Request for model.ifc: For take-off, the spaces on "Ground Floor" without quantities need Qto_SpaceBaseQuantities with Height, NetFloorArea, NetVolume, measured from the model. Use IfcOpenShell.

First a look at what the model holds.

```python
import ifcopenshell
import ifcopenshell.util.element
import ifcopenshell.util.unit

model = ifcopenshell.open("model.ifc")
print(model.schema)
for unit_type in ("LENGTHUNIT", "AREAUNIT", "VOLUMEUNIT"):
    print(unit_type, ifcopenshell.util.unit.calculate_unit_scale(model, unit_type))
storey = next(s for s in model.by_type("IfcBuildingStorey") if s.Name == "Ground Floor")
spaces = [e for e in ifcopenshell.util.element.get_decomposition(storey) if e.is_a("IfcSpace")]
for e in sorted(spaces, key=lambda e: e.id()):
    print(e.id(), e.is_a(), e.Name, list(ifcopenshell.util.element.get_psets(e, qtos_only=True)), sep=" | ")
```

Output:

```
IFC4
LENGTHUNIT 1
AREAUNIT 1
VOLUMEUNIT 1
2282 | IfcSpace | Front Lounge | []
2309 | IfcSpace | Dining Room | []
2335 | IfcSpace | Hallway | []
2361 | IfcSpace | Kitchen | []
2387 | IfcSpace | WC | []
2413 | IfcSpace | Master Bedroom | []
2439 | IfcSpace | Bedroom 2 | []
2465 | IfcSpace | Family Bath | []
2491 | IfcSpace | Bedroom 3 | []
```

```python
import ifcopenshell
import ifcopenshell.api.pset
import ifcopenshell.geom
import ifcopenshell.util.element
import ifcopenshell.util.shape
import ifcopenshell.util.unit

model = ifcopenshell.open("model.ifc")
unit_scale = ifcopenshell.util.unit.calculate_unit_scale(model)
area_scale = ifcopenshell.util.unit.calculate_unit_scale(model, "AREAUNIT")
volume_scale = ifcopenshell.util.unit.calculate_unit_scale(model, "VOLUMEUNIT")
settings = ifcopenshell.geom.settings()

storey = next(s for s in model.by_type("IfcBuildingStorey") if s.Name == "Ground Floor")
spaces = [e for e in ifcopenshell.util.element.get_decomposition(storey) if e.is_a("IfcSpace")]

for e in sorted(spaces, key=lambda e: e.id()):
    if ifcopenshell.util.element.get_psets(e, qtos_only=True, should_inherit=False):
        continue
    # Geometry comes back in metres, in the element's own axes.
    shape = ifcopenshell.geom.create_shape(settings, e)
    values = {
        "Height": ifcopenshell.util.shape.get_z(shape.geometry) / unit_scale,
        "NetFloorArea": ifcopenshell.util.shape.get_footprint_area(shape.geometry) / area_scale,
        "NetVolume": ifcopenshell.util.shape.get_volume(shape.geometry) / volume_scale,
    }
    qto = ifcopenshell.api.pset.add_qto(model, product=e, name="Qto_SpaceBaseQuantities")
    ifcopenshell.api.pset.edit_qto(model, qto=qto, properties=values)
    print(e.id(), {k: round(v, 3) for k, v in values.items()})

model.write("model_updated.ifc")
```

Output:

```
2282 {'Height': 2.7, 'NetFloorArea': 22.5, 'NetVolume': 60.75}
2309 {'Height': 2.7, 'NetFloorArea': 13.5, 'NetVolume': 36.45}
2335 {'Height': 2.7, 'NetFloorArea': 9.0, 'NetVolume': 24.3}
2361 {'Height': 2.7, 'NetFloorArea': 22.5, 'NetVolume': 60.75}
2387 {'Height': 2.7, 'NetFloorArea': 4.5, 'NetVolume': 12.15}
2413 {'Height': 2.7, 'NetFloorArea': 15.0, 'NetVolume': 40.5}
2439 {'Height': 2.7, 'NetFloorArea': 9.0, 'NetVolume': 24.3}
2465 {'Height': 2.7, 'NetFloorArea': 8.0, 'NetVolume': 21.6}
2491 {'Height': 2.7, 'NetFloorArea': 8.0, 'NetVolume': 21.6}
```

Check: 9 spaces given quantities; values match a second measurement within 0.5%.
